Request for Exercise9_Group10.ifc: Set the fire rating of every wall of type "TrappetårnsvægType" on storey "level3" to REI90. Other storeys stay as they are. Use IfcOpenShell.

First a look at what the model holds.

```python
import ifcopenshell
import ifcopenshell.util.element

model = ifcopenshell.open("Exercise9_Group10.ifc")
print(model.schema)
storey = next(s for s in model.by_type("IfcBuildingStorey") if s.Name == "level3")
walls = [e for e in ifcopenshell.util.element.get_decomposition(storey) if e.is_a("IfcWall")]
seen = {}
for e in walls:
    element_type = ifcopenshell.util.element.get_type(e)
    key = (element_type.Name if element_type != e and element_type else None, ifcopenshell.util.element.get_pset(e, "Pset_WallCommon", "FireRating"))
    seen[key] = seen.get(key, 0) + 1
for (name, value), count in sorted(seen.items(), key=str):
    print(count, "x", name, "|", value)
```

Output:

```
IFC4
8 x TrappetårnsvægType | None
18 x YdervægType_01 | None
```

```python
import ifcopenshell
import ifcopenshell.api.pset
import ifcopenshell.util.element

model = ifcopenshell.open("Exercise9_Group10.ifc")

storey = next(s for s in model.by_type("IfcBuildingStorey") if s.Name == "level3")
walls = [e for e in ifcopenshell.util.element.get_decomposition(storey) if e.is_a("IfcWall")]

count = 0
for e in walls:
    element_type = ifcopenshell.util.element.get_type(e)
    if element_type in (None, e) or element_type.Name != "TrappetårnsvægType":
        continue
    # add_pset returns the element's existing set when there is one.
    pset = ifcopenshell.api.pset.add_pset(model, product=e, name="Pset_WallCommon")
    ifcopenshell.api.pset.edit_pset(model, pset=pset, properties={"FireRating": "REI90"})
    count += 1

print(count, "walls updated")

model.write("Exercise9_Group10-out.ifc")
```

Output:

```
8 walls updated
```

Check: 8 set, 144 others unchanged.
